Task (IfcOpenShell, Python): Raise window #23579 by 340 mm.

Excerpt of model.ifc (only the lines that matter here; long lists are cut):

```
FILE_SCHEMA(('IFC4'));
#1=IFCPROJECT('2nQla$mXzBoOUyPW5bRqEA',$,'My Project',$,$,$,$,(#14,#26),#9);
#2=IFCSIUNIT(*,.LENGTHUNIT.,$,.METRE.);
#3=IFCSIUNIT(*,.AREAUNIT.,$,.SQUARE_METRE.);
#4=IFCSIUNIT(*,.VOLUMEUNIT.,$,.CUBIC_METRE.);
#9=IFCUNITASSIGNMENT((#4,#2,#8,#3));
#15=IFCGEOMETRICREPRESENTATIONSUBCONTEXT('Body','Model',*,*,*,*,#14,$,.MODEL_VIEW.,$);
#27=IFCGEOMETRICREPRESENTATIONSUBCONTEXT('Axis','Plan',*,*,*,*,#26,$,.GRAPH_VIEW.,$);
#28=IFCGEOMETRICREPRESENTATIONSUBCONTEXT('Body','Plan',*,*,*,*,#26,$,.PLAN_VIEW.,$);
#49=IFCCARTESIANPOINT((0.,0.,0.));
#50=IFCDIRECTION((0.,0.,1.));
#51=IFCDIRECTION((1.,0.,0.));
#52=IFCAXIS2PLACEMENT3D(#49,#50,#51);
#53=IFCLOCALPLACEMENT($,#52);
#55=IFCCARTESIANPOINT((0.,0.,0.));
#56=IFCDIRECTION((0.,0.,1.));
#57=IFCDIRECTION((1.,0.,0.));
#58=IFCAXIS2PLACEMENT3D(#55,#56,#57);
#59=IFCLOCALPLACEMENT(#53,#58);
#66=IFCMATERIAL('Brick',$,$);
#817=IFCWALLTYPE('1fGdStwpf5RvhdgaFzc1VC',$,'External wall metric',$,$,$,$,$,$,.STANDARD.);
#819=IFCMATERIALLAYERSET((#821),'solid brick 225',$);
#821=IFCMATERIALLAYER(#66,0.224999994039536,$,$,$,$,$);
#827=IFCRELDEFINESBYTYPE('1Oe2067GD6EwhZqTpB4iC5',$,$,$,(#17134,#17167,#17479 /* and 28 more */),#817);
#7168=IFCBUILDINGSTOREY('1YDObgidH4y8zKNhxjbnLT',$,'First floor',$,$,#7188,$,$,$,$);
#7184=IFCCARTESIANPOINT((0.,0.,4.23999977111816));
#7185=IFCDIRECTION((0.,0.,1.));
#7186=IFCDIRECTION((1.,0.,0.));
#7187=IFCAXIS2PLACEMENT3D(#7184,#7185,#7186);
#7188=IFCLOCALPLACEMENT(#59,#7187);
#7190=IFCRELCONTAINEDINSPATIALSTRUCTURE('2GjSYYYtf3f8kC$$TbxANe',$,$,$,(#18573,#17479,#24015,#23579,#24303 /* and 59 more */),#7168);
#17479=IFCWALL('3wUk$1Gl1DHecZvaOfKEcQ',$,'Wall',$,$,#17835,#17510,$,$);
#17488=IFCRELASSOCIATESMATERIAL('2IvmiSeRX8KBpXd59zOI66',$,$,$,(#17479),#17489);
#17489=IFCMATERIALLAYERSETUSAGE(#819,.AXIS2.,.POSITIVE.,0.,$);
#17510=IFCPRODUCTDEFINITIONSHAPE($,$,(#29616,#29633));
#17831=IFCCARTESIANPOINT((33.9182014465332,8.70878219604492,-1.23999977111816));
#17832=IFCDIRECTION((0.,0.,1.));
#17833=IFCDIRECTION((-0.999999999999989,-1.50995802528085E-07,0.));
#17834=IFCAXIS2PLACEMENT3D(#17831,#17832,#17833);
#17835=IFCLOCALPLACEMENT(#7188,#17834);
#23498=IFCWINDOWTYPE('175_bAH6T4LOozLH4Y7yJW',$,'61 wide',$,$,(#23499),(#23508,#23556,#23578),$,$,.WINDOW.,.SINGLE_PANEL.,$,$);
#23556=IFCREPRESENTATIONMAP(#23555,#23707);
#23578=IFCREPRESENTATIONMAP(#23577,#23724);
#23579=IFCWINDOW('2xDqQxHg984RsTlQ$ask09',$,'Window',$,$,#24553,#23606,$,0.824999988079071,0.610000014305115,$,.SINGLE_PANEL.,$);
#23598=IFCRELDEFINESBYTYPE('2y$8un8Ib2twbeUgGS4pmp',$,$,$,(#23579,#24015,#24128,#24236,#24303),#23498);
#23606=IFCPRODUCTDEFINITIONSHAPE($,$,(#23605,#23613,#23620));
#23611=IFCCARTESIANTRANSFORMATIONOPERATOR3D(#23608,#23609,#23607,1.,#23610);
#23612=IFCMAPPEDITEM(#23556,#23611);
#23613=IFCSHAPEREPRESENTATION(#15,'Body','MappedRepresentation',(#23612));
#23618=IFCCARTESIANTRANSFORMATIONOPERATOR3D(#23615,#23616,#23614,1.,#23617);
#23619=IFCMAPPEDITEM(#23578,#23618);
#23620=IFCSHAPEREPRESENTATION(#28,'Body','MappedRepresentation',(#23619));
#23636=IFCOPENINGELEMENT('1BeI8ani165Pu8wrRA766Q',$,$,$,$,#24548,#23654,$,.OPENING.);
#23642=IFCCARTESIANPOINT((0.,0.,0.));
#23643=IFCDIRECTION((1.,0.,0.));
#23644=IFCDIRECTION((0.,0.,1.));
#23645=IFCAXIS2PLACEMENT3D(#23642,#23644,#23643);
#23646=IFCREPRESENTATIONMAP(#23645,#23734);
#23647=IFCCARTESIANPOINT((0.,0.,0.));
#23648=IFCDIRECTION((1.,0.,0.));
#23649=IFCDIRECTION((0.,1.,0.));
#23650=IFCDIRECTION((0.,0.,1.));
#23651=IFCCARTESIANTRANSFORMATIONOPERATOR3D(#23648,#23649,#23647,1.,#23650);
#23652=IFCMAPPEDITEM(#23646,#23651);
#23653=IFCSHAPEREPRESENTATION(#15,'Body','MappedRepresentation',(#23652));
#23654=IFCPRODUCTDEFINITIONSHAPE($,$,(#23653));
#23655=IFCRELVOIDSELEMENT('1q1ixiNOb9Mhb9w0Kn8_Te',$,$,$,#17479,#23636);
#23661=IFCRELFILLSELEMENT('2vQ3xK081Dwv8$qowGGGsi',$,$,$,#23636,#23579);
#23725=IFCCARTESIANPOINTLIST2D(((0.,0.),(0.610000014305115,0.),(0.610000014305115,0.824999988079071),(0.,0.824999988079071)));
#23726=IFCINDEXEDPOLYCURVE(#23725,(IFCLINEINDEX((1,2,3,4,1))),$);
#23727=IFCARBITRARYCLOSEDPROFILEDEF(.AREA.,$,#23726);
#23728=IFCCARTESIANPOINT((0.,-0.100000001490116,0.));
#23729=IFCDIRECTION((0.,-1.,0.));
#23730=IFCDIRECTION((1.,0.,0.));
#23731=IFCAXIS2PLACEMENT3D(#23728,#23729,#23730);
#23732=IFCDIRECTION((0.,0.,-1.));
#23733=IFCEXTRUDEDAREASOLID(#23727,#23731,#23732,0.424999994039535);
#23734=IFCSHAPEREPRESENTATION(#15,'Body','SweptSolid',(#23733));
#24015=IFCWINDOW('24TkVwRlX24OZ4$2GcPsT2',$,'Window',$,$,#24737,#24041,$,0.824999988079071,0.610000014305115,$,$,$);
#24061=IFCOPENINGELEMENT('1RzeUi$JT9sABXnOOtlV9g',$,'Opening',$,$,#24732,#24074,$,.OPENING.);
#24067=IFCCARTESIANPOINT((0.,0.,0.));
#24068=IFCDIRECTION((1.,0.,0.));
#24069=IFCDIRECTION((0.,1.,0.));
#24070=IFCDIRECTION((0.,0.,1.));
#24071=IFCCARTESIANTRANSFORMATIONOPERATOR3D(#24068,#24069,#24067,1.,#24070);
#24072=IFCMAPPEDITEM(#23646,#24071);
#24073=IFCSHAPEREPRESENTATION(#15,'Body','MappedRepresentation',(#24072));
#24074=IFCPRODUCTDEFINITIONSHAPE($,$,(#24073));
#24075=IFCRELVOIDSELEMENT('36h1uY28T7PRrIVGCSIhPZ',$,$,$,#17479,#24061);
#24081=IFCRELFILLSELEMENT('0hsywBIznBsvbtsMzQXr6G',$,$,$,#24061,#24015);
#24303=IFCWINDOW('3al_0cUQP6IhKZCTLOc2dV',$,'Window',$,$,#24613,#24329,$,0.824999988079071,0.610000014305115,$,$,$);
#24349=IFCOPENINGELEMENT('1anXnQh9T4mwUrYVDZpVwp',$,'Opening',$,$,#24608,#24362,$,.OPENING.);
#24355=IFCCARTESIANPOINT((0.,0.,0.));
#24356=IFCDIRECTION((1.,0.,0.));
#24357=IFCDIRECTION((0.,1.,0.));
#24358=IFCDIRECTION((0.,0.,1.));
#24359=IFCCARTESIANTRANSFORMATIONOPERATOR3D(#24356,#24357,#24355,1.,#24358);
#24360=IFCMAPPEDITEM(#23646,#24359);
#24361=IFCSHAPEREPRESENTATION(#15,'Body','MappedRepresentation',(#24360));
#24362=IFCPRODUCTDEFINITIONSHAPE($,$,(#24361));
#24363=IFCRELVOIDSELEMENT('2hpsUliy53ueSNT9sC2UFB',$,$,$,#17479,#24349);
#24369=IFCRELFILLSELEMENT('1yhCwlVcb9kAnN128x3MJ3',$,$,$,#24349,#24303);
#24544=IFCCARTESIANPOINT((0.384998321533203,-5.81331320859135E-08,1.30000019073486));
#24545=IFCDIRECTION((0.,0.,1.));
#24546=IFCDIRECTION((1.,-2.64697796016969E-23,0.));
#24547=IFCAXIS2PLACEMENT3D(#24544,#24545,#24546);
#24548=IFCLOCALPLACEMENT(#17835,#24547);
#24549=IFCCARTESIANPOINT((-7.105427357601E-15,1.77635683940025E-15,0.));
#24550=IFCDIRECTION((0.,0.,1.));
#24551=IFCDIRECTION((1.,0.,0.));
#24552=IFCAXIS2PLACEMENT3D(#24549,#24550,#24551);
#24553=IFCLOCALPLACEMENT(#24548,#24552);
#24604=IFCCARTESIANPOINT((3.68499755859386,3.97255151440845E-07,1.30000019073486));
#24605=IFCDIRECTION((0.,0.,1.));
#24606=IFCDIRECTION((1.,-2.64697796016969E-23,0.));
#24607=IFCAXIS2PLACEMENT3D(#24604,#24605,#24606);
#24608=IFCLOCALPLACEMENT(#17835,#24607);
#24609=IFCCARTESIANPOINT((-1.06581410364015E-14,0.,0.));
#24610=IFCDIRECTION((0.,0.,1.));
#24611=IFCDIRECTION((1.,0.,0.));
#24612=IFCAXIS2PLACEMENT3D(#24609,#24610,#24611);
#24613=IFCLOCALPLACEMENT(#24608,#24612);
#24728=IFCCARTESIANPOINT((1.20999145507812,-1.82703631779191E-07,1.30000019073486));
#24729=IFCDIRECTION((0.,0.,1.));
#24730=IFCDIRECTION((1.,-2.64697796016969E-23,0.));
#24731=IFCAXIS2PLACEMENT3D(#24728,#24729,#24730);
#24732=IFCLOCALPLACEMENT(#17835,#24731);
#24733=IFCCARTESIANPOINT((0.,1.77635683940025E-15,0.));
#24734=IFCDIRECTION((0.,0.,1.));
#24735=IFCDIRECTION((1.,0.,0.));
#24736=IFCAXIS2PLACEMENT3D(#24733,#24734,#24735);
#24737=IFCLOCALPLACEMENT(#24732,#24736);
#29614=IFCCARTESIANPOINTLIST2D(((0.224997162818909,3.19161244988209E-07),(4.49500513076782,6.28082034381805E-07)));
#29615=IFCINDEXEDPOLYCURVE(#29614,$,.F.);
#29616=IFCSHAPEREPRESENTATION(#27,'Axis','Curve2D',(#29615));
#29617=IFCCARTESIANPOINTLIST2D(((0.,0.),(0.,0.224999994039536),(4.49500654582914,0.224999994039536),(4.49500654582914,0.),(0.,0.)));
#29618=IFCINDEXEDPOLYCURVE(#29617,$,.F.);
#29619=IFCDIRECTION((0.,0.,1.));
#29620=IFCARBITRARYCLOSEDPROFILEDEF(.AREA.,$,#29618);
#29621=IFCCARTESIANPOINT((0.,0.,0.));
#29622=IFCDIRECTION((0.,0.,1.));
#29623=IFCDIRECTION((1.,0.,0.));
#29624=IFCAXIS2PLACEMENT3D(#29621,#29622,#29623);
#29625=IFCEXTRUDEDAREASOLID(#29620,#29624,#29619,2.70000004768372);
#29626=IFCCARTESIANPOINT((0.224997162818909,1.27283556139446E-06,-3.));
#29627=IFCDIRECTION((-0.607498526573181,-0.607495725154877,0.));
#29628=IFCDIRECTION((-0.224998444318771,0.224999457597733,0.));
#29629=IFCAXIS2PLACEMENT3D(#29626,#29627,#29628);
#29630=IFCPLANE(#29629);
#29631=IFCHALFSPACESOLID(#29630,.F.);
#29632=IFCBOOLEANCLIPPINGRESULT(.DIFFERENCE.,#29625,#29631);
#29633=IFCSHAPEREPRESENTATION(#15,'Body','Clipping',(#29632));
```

```python
import numpy as np
import ifcopenshell
import ifcopenshell.api.geometry
import ifcopenshell.util.placement
import ifcopenshell.util.unit

model = ifcopenshell.open("model.ifc")
unit_scale = ifcopenshell.util.unit.calculate_unit_scale(model)

window = model.by_guid("2xDqQxHg984RsTlQ$ask09")
opening = window.FillsVoids[0].RelatingOpeningElement
dz = 0.34 / unit_scale

shift = np.array([0.0, 0.0, dz])
# The window is placed relative to its opening, so it follows when the opening moves.
matrix = ifcopenshell.util.placement.get_local_placement(opening.ObjectPlacement)
matrix[:3, 3] += shift
ifcopenshell.api.geometry.edit_object_placement(
    model, product=opening, matrix=matrix, is_si=False, should_transform_children=True
)

print(f"moved by {dz * unit_scale:+.3f} m")

model.write("model_rev.ifc")
```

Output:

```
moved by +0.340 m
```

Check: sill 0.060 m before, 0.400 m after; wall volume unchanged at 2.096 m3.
